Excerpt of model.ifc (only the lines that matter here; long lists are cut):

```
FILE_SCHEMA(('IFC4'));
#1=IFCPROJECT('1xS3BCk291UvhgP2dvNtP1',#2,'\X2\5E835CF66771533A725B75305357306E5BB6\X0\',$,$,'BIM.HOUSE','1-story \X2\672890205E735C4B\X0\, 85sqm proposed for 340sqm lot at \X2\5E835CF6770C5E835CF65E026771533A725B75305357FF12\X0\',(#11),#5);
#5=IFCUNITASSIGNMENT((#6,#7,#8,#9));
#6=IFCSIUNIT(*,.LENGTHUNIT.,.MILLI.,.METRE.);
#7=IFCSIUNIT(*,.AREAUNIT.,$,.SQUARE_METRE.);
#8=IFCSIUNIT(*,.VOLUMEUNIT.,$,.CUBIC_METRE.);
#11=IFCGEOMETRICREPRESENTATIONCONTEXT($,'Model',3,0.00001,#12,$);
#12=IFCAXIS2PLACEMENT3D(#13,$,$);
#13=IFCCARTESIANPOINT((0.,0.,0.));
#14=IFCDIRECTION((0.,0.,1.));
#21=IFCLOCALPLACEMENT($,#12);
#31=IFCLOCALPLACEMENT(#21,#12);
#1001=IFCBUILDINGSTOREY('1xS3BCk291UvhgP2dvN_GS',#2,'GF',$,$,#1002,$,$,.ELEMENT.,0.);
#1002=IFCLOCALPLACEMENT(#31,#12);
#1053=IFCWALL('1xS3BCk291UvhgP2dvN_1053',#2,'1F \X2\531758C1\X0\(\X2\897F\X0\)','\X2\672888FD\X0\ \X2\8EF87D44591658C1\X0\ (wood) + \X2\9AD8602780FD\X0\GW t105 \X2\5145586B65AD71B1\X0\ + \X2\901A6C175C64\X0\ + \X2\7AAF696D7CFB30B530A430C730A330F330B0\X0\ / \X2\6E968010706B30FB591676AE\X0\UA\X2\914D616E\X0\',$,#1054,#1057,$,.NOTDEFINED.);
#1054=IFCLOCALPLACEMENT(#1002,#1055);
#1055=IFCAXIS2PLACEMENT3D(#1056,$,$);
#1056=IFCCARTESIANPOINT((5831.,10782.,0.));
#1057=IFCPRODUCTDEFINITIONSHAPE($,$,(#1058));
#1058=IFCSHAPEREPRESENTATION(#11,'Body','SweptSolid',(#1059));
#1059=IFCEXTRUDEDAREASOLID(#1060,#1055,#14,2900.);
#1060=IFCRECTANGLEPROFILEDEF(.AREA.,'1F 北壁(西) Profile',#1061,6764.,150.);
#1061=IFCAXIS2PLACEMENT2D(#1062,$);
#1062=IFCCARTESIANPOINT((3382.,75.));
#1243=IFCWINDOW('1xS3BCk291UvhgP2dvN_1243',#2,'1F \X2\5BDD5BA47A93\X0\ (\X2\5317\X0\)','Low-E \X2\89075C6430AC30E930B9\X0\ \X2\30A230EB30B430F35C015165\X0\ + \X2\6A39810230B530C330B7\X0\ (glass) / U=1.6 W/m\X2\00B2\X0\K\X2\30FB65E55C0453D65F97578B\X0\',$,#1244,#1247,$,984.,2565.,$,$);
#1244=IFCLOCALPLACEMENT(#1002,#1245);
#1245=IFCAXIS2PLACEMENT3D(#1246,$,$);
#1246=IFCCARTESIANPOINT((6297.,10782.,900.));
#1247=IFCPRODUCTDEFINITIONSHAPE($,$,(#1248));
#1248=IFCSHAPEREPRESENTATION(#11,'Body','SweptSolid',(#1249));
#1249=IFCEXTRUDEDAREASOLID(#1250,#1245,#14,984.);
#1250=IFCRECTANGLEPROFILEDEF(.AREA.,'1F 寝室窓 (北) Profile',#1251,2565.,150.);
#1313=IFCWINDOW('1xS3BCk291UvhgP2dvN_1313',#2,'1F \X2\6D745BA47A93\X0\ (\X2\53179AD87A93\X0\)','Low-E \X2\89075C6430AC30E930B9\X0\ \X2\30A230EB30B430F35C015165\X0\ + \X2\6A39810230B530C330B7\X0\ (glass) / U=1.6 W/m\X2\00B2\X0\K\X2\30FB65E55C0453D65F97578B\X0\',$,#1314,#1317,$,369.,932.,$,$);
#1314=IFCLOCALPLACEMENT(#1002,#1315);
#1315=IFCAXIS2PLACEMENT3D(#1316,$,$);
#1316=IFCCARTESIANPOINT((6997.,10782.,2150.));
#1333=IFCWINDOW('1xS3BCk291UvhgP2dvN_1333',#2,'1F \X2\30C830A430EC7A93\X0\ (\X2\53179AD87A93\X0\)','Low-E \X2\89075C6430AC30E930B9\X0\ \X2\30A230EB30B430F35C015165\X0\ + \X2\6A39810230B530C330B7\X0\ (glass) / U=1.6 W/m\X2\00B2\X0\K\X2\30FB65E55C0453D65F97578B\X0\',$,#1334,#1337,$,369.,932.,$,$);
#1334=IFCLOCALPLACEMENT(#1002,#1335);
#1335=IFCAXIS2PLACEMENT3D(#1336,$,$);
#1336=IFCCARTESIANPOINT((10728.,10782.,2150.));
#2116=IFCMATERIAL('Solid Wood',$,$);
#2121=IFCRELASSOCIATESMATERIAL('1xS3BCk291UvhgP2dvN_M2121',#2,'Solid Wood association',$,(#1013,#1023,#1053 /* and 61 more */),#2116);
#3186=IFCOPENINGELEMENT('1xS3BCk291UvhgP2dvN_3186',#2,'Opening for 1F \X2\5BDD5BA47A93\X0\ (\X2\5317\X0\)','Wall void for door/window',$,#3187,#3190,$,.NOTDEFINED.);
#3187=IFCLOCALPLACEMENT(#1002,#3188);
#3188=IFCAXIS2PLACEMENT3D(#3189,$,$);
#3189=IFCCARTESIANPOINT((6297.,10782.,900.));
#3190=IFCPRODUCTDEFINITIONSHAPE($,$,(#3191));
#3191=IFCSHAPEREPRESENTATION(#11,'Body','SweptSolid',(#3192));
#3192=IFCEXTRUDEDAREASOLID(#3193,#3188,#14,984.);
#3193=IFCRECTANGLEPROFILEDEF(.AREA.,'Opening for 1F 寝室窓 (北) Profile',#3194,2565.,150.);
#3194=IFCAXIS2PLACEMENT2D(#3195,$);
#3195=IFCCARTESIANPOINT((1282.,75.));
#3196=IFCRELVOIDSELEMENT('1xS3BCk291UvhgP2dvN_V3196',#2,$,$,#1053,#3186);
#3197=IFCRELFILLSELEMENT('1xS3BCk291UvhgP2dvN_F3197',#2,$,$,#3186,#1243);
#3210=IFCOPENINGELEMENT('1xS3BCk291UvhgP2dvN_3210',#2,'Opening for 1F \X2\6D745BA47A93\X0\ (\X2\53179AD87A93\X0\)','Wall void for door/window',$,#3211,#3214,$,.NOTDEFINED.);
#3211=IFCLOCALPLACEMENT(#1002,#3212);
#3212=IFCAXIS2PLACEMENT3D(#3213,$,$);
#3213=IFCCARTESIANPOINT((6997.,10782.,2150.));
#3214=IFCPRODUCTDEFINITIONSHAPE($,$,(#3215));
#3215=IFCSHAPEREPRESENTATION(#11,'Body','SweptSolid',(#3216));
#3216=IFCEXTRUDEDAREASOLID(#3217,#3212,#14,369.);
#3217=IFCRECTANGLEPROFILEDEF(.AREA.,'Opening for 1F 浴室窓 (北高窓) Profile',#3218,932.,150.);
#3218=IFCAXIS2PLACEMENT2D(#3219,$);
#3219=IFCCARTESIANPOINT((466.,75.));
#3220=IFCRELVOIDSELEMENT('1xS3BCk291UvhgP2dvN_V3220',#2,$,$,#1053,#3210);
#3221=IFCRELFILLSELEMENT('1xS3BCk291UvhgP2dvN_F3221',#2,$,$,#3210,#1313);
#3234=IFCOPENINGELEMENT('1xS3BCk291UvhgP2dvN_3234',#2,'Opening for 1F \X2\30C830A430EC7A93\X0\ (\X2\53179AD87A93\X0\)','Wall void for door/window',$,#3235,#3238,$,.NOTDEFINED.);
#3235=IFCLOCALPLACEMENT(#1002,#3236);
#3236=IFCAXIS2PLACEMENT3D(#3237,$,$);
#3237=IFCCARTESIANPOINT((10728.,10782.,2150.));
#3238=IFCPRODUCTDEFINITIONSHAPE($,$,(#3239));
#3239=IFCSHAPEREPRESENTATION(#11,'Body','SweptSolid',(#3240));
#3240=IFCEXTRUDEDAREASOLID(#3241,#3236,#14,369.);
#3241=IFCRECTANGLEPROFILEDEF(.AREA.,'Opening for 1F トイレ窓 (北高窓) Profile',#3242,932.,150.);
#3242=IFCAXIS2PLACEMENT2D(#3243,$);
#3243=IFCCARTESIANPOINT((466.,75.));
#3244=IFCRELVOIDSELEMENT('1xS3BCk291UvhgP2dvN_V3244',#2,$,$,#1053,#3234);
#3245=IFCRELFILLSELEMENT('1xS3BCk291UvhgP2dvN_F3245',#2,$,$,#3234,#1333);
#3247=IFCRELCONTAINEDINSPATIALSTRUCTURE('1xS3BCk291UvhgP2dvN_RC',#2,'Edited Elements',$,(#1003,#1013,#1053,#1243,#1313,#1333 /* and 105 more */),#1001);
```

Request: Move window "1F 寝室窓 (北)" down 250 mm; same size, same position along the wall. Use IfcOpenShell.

```python
import numpy as np
import ifcopenshell
import ifcopenshell.api.geometry
import ifcopenshell.util.placement
import ifcopenshell.util.unit

model = ifcopenshell.open("model.ifc")
unit_scale = ifcopenshell.util.unit.calculate_unit_scale(model)

window = model.by_guid("1xS3BCk291UvhgP2dvN_1243")
opening = window.FillsVoids[0].RelatingOpeningElement
dz = -0.25 / unit_scale

shift = np.array([0.0, 0.0, dz])
# The window is not placed relative to its opening, so move both.
for product in (opening, window):
    matrix = ifcopenshell.util.placement.get_local_placement(product.ObjectPlacement)
    matrix[:3, 3] += shift
    ifcopenshell.api.geometry.edit_object_placement(model, product=product, matrix=matrix, is_si=False)

print(f"moved by {dz * unit_scale:+.3f} m")

model.write("model_updated.ifc")
```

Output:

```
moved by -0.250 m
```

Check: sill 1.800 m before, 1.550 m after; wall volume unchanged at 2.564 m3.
